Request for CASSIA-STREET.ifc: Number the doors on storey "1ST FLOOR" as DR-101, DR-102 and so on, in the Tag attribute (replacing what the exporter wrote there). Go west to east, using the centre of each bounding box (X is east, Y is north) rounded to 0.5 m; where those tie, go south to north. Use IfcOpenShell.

First a look at what the model holds.

```python
import ifcopenshell
import ifcopenshell.util.element
import ifcopenshell.util.placement

model = ifcopenshell.open("CASSIA-STREET.ifc")
print(model.schema)
storey = next(s for s in model.by_type("IfcBuildingStorey") if s.Name == "1ST FLOOR")
doors = [e for e in ifcopenshell.util.element.get_decomposition(storey) if e.is_a("IfcDoor")]
for e in sorted(doors, key=lambda e: e.id()):
    origin = ifcopenshell.util.placement.get_local_placement(e.ObjectPlacement)[:3, 3]
    print(e.id(), e.Tag, e.Name, origin.round(2) + 0.0, sep=" | ")
```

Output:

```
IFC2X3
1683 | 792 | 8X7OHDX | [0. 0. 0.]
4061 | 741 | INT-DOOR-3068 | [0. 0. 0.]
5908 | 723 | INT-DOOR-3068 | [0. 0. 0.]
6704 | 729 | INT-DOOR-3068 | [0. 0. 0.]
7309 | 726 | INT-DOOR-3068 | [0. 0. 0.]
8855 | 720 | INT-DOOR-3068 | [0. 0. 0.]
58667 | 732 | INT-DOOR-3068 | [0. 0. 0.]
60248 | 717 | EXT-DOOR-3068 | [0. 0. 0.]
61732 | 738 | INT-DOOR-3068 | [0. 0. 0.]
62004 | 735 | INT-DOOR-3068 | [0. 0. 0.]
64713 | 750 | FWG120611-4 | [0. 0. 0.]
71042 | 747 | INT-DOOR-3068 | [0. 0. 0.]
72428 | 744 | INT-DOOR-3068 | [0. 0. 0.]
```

```python
import ifcopenshell
import ifcopenshell.geom
import ifcopenshell.util.element
import ifcopenshell.util.shape

model = ifcopenshell.open("CASSIA-STREET.ifc")
settings = ifcopenshell.geom.settings()
settings.set("use-world-coords", True)


def centre(element):
    shape = ifcopenshell.geom.create_shape(settings, element)
    return ifcopenshell.util.shape.get_bbox_centroid(shape.geometry)


storey = next(s for s in model.by_type("IfcBuildingStorey") if s.Name == "1ST FLOOR")
doors = [e for e in ifcopenshell.util.element.get_decomposition(storey) if e.is_a("IfcDoor")]

# Insertion points can sit at a corner or the storey origin, so sort by the geometry (in metres).
centres = {e: centre(e) for e in doors}
doors.sort(key=lambda e: (round(centres[e][0] / 0.5), centres[e][1]))

for i, e in enumerate(doors, start=1):
    number = f"DR-1{i:02d}"
    e.Tag = number
    print(e.id(), number)

model.write("CASSIA-STREET-out.ifc")
```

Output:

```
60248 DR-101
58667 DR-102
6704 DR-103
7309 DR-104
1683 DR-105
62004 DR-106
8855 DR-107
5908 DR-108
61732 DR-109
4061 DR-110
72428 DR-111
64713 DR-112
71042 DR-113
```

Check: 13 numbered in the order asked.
